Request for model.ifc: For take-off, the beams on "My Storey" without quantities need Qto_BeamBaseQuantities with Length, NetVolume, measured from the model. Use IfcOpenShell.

First a look at what the model holds.

```python
import ifcopenshell
import ifcopenshell.util.element
import ifcopenshell.util.unit

model = ifcopenshell.open("model.ifc")
print(model.schema)
for unit_type in ("LENGTHUNIT", "AREAUNIT", "VOLUMEUNIT"):
    print(unit_type, ifcopenshell.util.unit.calculate_unit_scale(model, unit_type))
storey = next(s for s in model.by_type("IfcBuildingStorey") if s.Name == "My Storey")
beams = [e for e in ifcopenshell.util.element.get_decomposition(storey) if e.is_a("IfcBeam")]
for e in sorted(beams, key=lambda e: e.id()):
    print(e.id(), e.is_a(), e.Name, list(ifcopenshell.util.element.get_psets(e, qtos_only=True)), sep=" | ")
```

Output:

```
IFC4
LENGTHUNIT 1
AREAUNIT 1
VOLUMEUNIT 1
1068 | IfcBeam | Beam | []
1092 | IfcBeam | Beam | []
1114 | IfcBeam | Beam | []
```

```python
import ifcopenshell
import ifcopenshell.api.pset
import ifcopenshell.geom
import ifcopenshell.util.element
import ifcopenshell.util.shape
import ifcopenshell.util.unit

model = ifcopenshell.open("model.ifc")
unit_scale = ifcopenshell.util.unit.calculate_unit_scale(model)
volume_scale = ifcopenshell.util.unit.calculate_unit_scale(model, "VOLUMEUNIT")
settings = ifcopenshell.geom.settings()

storey = next(s for s in model.by_type("IfcBuildingStorey") if s.Name == "My Storey")
beams = [e for e in ifcopenshell.util.element.get_decomposition(storey) if e.is_a("IfcBeam")]

for e in sorted(beams, key=lambda e: e.id()):
    if ifcopenshell.util.element.get_psets(e, qtos_only=True, should_inherit=False):
        continue
    # Geometry comes back in metres, in the element's own axes.
    shape = ifcopenshell.geom.create_shape(settings, e)
    values = {
        "Length": ifcopenshell.util.shape.get_max_xyz(shape.geometry) / unit_scale,
        "NetVolume": ifcopenshell.util.shape.get_volume(shape.geometry) / volume_scale,
    }
    qto = ifcopenshell.api.pset.add_qto(model, product=e, name="Qto_BeamBaseQuantities")
    ifcopenshell.api.pset.edit_qto(model, qto=qto, properties=values)
    print(e.id(), {k: round(v, 3) for k, v in values.items()})

model.write("model_v2.ifc")
```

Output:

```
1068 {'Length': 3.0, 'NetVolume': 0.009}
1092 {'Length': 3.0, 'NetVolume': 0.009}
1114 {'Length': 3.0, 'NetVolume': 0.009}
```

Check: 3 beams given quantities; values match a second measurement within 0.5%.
